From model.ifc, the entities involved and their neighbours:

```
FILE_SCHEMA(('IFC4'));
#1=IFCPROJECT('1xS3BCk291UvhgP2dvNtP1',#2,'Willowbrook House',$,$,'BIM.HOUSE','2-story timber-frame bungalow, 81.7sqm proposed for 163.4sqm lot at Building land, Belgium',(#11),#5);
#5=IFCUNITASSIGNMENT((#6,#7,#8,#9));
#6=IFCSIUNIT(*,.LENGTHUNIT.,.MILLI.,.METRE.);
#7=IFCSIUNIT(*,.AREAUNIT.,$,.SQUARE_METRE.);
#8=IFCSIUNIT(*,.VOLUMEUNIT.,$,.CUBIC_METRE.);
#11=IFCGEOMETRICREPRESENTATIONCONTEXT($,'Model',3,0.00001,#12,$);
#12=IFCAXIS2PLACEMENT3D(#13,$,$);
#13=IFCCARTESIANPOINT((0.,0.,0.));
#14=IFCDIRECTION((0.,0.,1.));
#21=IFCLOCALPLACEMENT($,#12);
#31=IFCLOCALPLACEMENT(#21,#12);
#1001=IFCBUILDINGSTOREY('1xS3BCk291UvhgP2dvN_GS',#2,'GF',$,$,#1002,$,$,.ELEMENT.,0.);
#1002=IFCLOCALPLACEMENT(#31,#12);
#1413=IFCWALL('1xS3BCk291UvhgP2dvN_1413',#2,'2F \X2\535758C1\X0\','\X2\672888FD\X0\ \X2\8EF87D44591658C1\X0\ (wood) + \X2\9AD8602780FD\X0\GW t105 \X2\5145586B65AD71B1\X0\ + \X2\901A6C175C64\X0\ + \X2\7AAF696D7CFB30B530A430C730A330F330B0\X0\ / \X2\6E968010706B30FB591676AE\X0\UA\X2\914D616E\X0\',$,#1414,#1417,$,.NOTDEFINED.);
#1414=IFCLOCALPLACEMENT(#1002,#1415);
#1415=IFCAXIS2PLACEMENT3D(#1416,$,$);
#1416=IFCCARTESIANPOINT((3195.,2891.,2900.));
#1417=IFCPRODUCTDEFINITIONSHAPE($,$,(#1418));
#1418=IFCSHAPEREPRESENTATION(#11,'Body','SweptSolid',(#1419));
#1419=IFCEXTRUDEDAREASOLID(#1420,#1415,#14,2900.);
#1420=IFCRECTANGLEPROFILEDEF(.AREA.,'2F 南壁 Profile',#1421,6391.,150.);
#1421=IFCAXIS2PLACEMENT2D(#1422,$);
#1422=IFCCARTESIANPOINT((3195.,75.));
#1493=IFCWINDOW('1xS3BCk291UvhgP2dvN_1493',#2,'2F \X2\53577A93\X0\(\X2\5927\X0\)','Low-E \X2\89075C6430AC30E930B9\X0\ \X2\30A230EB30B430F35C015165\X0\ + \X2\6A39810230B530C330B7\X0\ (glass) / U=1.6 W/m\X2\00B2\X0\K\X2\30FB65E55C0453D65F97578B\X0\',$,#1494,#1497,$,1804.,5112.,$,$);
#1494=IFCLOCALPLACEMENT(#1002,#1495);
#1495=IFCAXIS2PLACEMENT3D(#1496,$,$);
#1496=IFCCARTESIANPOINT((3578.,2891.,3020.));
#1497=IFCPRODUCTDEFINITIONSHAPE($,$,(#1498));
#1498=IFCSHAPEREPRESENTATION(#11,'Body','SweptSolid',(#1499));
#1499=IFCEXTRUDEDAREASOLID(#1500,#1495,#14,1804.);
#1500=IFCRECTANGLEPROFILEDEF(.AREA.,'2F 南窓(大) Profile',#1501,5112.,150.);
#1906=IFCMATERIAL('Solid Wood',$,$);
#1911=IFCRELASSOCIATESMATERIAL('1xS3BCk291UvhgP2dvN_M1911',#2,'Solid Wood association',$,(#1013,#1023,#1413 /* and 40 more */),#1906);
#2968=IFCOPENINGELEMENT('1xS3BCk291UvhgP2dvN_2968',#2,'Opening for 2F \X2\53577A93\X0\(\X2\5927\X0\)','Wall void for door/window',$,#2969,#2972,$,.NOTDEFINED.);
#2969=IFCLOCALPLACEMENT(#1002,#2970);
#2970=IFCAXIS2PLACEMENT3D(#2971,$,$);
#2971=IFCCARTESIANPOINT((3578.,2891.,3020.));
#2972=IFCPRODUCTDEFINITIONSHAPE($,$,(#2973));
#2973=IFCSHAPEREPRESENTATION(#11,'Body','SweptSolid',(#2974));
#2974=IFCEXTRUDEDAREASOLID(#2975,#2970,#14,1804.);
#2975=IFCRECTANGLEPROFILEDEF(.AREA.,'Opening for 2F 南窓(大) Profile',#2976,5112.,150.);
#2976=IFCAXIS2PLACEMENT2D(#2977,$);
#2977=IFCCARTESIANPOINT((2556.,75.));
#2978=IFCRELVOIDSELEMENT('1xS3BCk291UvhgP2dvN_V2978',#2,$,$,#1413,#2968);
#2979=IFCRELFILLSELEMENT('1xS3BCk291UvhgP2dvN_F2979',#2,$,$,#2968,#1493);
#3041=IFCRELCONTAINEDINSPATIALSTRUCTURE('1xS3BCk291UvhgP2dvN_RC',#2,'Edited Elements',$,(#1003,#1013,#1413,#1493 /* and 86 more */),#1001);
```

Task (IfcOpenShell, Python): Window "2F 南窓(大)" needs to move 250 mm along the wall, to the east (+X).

```python
import ifcopenshell
import ifcopenshell.api.geometry
import ifcopenshell.util.placement
import ifcopenshell.util.unit

model = ifcopenshell.open("model.ifc")
unit_scale = ifcopenshell.util.unit.calculate_unit_scale(model)

window = model.by_guid("1xS3BCk291UvhgP2dvN_1493")
opening = window.FillsVoids[0].RelatingOpeningElement
wall = opening.VoidsElements[0].RelatingBuildingElement

wall_matrix = ifcopenshell.util.placement.get_local_placement(wall.ObjectPlacement)
shift = wall_matrix[:3, 0] * 0.25 / unit_scale
before = ifcopenshell.util.placement.get_local_placement(window.ObjectPlacement)[:3, 3].copy()

# The window is not placed relative to its opening, so move both.
for product in (opening, window):
    matrix = ifcopenshell.util.placement.get_local_placement(product.ObjectPlacement)
    matrix[:3, 3] += shift
    ifcopenshell.api.geometry.edit_object_placement(model, product=product, matrix=matrix, is_si=False)

after = ifcopenshell.util.placement.get_local_placement(window.ObjectPlacement)[:3, 3]
print("window moved by", (after - before).round(3) + 0.0)

model.write("model_edited.ifc")
```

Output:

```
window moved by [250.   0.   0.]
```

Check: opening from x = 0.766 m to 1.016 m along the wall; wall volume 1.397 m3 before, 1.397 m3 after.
